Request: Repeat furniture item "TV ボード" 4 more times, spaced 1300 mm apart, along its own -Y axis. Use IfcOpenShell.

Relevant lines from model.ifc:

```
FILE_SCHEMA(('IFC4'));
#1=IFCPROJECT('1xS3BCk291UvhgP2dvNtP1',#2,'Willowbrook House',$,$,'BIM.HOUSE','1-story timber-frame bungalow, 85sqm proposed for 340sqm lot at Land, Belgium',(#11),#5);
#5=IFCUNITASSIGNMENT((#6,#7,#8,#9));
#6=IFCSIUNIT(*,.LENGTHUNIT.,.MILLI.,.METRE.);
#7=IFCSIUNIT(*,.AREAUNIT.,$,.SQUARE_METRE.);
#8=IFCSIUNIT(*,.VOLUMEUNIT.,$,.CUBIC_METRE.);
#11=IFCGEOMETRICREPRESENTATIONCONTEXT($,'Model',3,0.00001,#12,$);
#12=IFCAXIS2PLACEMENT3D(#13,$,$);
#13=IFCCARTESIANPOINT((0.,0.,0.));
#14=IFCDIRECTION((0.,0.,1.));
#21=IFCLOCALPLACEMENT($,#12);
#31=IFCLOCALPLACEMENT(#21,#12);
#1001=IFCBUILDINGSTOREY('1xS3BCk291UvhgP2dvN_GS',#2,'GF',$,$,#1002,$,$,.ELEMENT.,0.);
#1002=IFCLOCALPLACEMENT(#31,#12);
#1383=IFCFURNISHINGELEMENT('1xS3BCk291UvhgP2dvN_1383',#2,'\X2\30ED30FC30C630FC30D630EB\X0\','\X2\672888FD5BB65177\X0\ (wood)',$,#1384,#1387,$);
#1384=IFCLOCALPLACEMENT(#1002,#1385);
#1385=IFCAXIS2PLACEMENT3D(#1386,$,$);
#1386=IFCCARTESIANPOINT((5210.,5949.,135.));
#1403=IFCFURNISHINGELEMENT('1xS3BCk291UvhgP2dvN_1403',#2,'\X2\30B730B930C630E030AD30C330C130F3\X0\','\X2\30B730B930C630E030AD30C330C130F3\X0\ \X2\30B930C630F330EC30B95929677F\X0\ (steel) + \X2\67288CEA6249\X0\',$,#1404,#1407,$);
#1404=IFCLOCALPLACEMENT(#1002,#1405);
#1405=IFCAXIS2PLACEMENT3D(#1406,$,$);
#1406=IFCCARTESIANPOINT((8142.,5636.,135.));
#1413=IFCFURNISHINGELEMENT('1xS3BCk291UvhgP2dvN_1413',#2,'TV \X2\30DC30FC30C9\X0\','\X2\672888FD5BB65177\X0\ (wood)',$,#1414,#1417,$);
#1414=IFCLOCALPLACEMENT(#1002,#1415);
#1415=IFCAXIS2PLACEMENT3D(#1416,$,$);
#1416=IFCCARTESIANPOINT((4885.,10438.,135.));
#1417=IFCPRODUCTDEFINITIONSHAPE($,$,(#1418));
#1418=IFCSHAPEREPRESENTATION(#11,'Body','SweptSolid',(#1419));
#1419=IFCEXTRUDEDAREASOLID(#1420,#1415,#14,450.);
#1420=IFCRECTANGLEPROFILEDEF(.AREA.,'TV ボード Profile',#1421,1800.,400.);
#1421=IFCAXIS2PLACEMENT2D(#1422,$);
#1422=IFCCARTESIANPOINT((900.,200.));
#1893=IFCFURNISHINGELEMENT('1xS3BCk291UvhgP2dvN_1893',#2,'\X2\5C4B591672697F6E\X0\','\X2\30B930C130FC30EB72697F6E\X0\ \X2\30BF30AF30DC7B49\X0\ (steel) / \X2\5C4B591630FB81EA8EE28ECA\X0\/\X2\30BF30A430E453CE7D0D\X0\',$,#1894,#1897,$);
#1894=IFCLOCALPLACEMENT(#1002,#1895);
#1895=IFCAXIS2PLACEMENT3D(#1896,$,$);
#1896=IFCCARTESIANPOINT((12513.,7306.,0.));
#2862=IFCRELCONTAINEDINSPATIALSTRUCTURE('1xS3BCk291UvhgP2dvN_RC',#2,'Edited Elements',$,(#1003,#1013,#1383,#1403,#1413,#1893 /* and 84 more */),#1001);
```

```python
import ifcopenshell
import ifcopenshell.api.geometry
import ifcopenshell.api.root
import ifcopenshell.util.element
import ifcopenshell.util.placement

model = ifcopenshell.open("model.ifc")


def reuse_history(source, copy):
    """copy_class also copies each property set's owner history, people and application; keep the originals."""
    for rel in copy.IsDefinedBy:
        if rel.is_a("IfcRelDefinesByProperties") and (history := rel.RelatingPropertyDefinition.OwnerHistory):
            rel.RelatingPropertyDefinition.OwnerHistory = source.OwnerHistory
            ifcopenshell.util.element.remove_deep2(model, history)


source = model.by_guid("1xS3BCk291UvhgP2dvN_1413")
base = ifcopenshell.util.placement.get_local_placement(source.ObjectPlacement)
step = -base[:3, 1] * 1300.0

for i in range(1, 5):
    copy = ifcopenshell.api.root.copy_class(model, product=source)
    copy.Representation = ifcopenshell.util.element.copy_deep(
        model, source.Representation, exclude=["IfcGeometricRepresentationContext", "IfcRepresentationMap"]
    )
    reuse_history(source, copy)
    matrix = base.copy()
    matrix[:3, 3] += i * step
    print("added at", matrix[:3, 3].round(3) + 0.0)
    ifcopenshell.api.geometry.edit_object_placement(model, product=copy, matrix=matrix, is_si=False)

model.write("model_rev.ifc")
```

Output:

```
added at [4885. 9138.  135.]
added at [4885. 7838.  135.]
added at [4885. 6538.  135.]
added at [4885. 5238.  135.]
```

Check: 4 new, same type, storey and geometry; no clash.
